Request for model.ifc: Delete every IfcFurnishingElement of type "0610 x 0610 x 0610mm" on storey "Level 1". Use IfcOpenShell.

First a look at what the model holds.

```python
import ifcopenshell
import ifcopenshell.util.element

model = ifcopenshell.open("model.ifc")
print(model.schema)
storey = next(s for s in model.by_type("IfcBuildingStorey") if s.Name == "Level 1")
furniture = [e for e in ifcopenshell.util.element.get_decomposition(storey) if e.is_a("IfcFurnishingElement")]
seen = {}
for e in furniture:
    element_type = ifcopenshell.util.element.get_type(e)
    name = element_type.Name if element_type not in (None, e) else None
    seen[name] = seen.get(name, 0) + 1
for name, count in sorted(seen.items(), key=str):
    print(count, "x", name)
```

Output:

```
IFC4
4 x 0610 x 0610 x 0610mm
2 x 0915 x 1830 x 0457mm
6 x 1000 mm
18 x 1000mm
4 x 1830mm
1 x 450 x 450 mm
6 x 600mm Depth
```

```python
import ifcopenshell
import ifcopenshell.api.root
import ifcopenshell.util.element

model = ifcopenshell.open("model.ifc")

storey = next(s for s in model.by_type("IfcBuildingStorey") if s.Name == "Level 1")
furniture = [e for e in ifcopenshell.util.element.get_decomposition(storey) if e.is_a("IfcFurnishingElement")]
targets = [e for e in furniture if (t := ifcopenshell.util.element.get_type(e)) not in (None, e) and t.Name == "0610 x 0610 x 0610mm"]

for e in targets:
    ifcopenshell.api.root.remove_product(model, product=e)
print(len(targets), "removed")

model.write("model_v2.ifc")
```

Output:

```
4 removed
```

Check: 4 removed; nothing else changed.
